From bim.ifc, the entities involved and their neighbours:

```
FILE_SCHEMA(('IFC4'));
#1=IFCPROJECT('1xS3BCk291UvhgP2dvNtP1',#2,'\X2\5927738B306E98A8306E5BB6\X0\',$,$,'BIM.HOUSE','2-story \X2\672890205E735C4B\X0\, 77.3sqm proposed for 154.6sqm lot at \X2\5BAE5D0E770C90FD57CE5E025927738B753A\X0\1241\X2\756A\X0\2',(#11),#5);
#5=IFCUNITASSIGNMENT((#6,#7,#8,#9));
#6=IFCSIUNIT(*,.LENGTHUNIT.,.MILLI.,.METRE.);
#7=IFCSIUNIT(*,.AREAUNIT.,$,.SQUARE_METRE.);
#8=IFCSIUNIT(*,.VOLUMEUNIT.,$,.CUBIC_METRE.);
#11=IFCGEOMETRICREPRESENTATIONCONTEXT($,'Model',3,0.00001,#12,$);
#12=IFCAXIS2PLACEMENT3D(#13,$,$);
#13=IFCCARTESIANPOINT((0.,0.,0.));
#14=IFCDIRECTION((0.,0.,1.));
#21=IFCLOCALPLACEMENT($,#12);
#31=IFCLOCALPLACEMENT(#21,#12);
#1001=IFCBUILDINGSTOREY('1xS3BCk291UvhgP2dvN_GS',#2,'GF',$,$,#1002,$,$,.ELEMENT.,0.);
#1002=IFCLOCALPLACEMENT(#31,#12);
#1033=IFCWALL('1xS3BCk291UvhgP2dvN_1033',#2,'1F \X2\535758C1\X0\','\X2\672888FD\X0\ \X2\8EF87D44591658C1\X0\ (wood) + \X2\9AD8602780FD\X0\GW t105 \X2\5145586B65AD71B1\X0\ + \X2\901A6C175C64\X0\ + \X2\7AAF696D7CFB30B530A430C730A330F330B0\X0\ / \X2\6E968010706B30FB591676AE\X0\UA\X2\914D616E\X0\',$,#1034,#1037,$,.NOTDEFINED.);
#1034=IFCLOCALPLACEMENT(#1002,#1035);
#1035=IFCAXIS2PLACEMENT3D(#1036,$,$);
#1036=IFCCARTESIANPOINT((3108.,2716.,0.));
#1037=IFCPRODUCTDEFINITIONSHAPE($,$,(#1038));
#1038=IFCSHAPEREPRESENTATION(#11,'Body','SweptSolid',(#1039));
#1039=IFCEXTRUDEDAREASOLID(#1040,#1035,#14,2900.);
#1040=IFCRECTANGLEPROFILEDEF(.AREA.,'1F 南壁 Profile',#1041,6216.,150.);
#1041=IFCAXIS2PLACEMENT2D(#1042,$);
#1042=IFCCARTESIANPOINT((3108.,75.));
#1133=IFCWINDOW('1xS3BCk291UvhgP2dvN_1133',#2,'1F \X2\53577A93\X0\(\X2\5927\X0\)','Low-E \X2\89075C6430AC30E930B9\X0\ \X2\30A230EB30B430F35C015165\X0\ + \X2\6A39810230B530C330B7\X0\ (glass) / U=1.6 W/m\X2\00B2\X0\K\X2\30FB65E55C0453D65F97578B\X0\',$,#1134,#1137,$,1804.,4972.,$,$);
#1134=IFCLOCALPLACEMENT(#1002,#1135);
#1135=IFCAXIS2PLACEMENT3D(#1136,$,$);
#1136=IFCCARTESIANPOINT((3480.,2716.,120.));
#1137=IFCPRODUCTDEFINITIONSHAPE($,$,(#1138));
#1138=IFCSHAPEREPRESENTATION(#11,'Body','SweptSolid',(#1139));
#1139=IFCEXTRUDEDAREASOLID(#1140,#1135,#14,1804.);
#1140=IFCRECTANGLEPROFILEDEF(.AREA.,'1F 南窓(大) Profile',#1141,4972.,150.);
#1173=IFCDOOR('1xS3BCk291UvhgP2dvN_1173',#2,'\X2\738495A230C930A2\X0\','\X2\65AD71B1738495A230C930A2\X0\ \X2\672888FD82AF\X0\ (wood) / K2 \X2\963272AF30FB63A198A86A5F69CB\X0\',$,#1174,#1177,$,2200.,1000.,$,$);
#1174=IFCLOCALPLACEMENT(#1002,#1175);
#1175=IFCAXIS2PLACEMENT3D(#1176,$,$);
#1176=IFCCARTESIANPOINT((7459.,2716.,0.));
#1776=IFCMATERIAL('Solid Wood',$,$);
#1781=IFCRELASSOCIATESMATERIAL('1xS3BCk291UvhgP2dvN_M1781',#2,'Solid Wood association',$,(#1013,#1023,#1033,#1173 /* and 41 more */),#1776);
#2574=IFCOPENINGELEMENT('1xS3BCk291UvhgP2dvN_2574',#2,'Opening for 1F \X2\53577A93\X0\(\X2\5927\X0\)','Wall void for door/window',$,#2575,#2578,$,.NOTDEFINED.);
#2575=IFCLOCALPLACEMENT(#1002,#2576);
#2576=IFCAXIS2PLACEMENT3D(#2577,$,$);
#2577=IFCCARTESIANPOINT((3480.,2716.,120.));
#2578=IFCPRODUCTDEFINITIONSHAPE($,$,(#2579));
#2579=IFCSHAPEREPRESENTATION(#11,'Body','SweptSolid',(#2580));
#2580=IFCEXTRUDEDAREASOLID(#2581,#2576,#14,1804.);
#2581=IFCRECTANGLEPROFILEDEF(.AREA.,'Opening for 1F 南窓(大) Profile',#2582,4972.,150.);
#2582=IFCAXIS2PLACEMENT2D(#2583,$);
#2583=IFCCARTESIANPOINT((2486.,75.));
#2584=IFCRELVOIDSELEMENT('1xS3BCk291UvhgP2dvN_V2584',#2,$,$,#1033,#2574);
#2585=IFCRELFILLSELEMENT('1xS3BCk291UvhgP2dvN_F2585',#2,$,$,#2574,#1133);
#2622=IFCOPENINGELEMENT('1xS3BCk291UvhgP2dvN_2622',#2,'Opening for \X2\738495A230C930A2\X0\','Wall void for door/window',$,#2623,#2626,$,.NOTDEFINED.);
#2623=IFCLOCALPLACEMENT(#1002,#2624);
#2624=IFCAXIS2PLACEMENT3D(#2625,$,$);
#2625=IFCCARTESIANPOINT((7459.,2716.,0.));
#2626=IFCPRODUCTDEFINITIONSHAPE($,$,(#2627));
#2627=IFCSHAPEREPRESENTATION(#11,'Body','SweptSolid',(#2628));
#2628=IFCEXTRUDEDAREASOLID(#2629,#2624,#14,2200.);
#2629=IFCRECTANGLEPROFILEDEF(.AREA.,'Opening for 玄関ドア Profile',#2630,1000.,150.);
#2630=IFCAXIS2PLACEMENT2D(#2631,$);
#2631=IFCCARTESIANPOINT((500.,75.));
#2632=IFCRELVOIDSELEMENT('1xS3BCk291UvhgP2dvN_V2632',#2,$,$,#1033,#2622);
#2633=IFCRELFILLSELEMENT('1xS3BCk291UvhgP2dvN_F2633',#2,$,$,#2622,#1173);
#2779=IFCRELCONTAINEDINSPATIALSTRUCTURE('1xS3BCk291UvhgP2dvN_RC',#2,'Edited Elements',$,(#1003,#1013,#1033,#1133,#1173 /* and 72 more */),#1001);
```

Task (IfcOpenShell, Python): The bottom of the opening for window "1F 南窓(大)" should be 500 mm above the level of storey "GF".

```python
import numpy as np
import ifcopenshell
import ifcopenshell.api.geometry
import ifcopenshell.geom
import ifcopenshell.util.element
import ifcopenshell.util.placement
import ifcopenshell.util.shape
import ifcopenshell.util.unit

model = ifcopenshell.open("bim.ifc")
unit_scale = ifcopenshell.util.unit.calculate_unit_scale(model)

window = model.by_guid("1xS3BCk291UvhgP2dvN_1133")
opening = window.FillsVoids[0].RelatingOpeningElement
storey = ifcopenshell.util.element.get_container(window, ifc_class="IfcBuildingStorey")
level = ifcopenshell.util.placement.get_local_placement(storey.ObjectPlacement)[2, 3]

# The opening's origin need not be at the sill, so measure its lowest point.
shape = ifcopenshell.geom.create_shape(ifcopenshell.geom.settings(), opening)
bottom = ifcopenshell.util.shape.get_shape_bottom_elevation(shape, shape.geometry) / unit_scale
dz = level + 500.0 - bottom

shift = np.array([0.0, 0.0, dz])
# The window is not placed relative to its opening, so move both.
for product in (opening, window):
    matrix = ifcopenshell.util.placement.get_local_placement(product.ObjectPlacement)
    matrix[:3, 3] += shift
    ifcopenshell.api.geometry.edit_object_placement(model, product=product, matrix=matrix, is_si=False)

print(f"moved by {dz * unit_scale:+.3f} m")

model.write("bim-out.ifc")
```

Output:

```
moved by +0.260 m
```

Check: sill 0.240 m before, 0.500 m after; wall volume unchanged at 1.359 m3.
